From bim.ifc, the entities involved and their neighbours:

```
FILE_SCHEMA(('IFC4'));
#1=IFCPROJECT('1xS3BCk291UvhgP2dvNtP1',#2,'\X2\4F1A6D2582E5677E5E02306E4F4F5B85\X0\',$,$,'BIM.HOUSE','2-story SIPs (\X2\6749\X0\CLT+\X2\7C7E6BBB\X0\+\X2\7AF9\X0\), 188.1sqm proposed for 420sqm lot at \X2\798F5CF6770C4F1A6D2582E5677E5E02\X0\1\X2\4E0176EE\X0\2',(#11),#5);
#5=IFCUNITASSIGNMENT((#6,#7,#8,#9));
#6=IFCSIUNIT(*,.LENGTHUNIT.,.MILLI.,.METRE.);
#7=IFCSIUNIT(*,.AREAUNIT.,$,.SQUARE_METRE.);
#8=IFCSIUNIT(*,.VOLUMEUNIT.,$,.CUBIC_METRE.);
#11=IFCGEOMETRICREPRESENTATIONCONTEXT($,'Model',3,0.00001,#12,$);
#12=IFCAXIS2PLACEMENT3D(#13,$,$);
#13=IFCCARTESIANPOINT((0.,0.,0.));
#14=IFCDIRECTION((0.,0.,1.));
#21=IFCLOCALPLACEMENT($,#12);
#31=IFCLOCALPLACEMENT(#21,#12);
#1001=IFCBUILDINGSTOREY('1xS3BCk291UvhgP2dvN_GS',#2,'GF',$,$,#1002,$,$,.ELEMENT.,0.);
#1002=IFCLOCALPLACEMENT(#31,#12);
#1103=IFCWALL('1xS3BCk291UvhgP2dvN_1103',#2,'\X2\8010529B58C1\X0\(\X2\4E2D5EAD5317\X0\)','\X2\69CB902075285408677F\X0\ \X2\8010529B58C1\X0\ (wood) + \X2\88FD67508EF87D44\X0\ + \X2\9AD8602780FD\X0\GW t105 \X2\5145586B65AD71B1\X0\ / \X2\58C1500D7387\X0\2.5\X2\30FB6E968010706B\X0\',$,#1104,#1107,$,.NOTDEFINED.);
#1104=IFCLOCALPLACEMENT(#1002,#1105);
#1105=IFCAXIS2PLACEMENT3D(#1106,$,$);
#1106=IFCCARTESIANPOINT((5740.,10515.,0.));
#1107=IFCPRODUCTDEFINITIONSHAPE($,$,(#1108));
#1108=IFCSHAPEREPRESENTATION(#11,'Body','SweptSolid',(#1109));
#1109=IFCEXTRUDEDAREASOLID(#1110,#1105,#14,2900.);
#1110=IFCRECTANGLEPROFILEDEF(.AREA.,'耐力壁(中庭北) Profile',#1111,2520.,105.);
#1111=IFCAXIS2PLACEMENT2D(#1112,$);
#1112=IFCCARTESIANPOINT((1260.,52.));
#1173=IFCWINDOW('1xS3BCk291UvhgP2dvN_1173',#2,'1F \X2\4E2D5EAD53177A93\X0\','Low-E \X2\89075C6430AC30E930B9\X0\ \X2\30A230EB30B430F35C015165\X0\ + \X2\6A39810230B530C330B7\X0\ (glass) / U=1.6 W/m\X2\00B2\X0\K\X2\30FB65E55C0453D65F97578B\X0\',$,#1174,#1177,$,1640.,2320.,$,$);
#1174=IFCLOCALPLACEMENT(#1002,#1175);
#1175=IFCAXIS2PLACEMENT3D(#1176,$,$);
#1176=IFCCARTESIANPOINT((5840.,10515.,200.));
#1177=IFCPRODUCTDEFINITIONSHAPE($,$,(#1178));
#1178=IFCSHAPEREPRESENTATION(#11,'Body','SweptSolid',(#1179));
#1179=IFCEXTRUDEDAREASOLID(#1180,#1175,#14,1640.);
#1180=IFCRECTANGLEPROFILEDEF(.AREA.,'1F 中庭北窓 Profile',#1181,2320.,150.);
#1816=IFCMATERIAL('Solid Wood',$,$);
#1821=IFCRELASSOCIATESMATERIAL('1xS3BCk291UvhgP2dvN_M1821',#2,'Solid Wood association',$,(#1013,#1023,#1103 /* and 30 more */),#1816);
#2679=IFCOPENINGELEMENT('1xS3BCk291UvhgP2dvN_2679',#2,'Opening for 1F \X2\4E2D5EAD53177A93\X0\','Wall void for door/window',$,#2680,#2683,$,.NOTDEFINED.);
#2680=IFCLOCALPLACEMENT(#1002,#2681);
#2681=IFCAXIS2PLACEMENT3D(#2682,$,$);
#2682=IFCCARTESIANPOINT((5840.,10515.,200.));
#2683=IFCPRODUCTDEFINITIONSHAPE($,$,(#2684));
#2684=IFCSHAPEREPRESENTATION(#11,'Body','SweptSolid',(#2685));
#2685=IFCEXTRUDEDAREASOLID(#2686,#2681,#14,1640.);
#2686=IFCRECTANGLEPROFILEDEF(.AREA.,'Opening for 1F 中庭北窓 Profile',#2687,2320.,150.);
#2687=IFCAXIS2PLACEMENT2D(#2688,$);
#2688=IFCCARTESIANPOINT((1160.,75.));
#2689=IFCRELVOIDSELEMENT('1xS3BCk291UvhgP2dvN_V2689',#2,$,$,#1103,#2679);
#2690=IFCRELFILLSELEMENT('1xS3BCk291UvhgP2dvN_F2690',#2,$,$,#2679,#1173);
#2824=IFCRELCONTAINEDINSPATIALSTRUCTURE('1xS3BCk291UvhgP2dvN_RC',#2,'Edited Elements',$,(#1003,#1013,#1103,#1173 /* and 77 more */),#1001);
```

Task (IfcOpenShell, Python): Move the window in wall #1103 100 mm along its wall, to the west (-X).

```python
import ifcopenshell
import ifcopenshell.api.geometry
import ifcopenshell.util.placement

model = ifcopenshell.open("bim.ifc")

window = model.by_id(1173)
opening = window.FillsVoids[0].RelatingOpeningElement
wall = opening.VoidsElements[0].RelatingBuildingElement

wall_matrix = ifcopenshell.util.placement.get_local_placement(wall.ObjectPlacement)
shift = wall_matrix[:3, 0] * -100.0
before = ifcopenshell.util.placement.get_local_placement(window.ObjectPlacement)[:3, 3].copy()

# The window is not placed relative to its opening, so move both.
for product in (opening, window):
    matrix = ifcopenshell.util.placement.get_local_placement(product.ObjectPlacement)
    matrix[:3, 3] += shift
    ifcopenshell.api.geometry.edit_object_placement(model, product=product, matrix=matrix, is_si=False)

after = ifcopenshell.util.placement.get_local_placement(window.ObjectPlacement)[:3, 3]
print("window moved by", (after - before).round(3) + 0.0)

model.write("bim_v2.ifc")
```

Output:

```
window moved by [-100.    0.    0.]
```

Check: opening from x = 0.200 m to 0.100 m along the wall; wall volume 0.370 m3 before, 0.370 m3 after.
